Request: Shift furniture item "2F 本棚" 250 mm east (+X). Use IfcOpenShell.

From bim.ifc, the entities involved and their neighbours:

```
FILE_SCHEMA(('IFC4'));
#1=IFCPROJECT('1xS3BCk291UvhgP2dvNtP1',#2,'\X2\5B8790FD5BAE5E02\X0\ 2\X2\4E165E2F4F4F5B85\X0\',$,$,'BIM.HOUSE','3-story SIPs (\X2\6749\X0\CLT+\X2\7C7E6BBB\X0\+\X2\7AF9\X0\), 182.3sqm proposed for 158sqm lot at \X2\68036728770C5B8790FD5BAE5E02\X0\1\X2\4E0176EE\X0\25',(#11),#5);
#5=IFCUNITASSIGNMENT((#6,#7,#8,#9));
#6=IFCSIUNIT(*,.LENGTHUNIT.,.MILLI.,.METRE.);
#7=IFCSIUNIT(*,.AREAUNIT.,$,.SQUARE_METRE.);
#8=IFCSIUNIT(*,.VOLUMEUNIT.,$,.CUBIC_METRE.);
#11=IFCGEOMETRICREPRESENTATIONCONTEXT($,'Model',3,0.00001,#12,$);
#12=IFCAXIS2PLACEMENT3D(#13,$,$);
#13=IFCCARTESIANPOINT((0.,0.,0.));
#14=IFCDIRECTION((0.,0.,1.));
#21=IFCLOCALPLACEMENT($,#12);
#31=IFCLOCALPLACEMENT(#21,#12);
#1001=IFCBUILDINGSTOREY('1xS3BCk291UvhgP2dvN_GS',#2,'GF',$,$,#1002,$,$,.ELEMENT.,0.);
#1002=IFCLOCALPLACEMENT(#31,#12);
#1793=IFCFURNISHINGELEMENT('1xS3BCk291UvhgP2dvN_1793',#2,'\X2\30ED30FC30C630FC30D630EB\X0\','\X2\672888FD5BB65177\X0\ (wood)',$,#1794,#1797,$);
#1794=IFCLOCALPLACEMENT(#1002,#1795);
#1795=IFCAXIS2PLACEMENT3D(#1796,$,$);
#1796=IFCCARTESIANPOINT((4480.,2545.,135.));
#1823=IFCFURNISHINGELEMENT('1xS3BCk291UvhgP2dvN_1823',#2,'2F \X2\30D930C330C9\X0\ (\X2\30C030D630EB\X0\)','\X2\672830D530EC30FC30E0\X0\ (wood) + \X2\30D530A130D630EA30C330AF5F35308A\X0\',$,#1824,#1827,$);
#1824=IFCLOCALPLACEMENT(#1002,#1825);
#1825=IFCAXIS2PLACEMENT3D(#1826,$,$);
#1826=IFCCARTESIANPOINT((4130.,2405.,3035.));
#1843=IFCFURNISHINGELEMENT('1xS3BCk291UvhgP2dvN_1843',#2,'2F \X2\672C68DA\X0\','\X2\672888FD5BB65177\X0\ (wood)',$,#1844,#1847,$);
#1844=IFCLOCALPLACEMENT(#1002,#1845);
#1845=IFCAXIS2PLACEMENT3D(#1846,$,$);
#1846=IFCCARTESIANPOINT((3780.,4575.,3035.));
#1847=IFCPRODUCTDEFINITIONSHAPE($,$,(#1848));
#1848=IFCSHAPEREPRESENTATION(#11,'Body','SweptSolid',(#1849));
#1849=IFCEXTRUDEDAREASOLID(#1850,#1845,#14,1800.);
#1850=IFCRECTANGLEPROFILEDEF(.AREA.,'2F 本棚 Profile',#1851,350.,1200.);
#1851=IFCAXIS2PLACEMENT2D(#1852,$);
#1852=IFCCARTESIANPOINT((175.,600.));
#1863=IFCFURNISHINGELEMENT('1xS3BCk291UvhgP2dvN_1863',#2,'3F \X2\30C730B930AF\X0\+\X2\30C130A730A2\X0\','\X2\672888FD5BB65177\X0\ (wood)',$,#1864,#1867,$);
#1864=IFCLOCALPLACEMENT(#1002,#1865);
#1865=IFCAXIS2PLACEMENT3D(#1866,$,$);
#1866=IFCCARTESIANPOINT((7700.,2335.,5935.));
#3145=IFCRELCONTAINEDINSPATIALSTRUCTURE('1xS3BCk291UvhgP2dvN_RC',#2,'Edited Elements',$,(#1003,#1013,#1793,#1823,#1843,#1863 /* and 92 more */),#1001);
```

```python
import ifcopenshell
import ifcopenshell.api.geometry
import ifcopenshell.util.placement

model = ifcopenshell.open("bim.ifc")

item = model.by_guid("1xS3BCk291UvhgP2dvN_1843")
matrix = ifcopenshell.util.placement.get_local_placement(item.ObjectPlacement)
matrix[0, 3] += 250.0
ifcopenshell.api.geometry.edit_object_placement(model, product=item, matrix=matrix, is_si=False)

print(ifcopenshell.util.placement.get_local_placement(item.ObjectPlacement).round(3) + 0.0)

model.write("bim_v2.ifc")
```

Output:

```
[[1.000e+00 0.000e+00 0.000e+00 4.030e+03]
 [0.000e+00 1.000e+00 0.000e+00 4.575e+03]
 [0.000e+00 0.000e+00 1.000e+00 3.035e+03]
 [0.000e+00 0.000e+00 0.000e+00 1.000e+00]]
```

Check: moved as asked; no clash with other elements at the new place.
